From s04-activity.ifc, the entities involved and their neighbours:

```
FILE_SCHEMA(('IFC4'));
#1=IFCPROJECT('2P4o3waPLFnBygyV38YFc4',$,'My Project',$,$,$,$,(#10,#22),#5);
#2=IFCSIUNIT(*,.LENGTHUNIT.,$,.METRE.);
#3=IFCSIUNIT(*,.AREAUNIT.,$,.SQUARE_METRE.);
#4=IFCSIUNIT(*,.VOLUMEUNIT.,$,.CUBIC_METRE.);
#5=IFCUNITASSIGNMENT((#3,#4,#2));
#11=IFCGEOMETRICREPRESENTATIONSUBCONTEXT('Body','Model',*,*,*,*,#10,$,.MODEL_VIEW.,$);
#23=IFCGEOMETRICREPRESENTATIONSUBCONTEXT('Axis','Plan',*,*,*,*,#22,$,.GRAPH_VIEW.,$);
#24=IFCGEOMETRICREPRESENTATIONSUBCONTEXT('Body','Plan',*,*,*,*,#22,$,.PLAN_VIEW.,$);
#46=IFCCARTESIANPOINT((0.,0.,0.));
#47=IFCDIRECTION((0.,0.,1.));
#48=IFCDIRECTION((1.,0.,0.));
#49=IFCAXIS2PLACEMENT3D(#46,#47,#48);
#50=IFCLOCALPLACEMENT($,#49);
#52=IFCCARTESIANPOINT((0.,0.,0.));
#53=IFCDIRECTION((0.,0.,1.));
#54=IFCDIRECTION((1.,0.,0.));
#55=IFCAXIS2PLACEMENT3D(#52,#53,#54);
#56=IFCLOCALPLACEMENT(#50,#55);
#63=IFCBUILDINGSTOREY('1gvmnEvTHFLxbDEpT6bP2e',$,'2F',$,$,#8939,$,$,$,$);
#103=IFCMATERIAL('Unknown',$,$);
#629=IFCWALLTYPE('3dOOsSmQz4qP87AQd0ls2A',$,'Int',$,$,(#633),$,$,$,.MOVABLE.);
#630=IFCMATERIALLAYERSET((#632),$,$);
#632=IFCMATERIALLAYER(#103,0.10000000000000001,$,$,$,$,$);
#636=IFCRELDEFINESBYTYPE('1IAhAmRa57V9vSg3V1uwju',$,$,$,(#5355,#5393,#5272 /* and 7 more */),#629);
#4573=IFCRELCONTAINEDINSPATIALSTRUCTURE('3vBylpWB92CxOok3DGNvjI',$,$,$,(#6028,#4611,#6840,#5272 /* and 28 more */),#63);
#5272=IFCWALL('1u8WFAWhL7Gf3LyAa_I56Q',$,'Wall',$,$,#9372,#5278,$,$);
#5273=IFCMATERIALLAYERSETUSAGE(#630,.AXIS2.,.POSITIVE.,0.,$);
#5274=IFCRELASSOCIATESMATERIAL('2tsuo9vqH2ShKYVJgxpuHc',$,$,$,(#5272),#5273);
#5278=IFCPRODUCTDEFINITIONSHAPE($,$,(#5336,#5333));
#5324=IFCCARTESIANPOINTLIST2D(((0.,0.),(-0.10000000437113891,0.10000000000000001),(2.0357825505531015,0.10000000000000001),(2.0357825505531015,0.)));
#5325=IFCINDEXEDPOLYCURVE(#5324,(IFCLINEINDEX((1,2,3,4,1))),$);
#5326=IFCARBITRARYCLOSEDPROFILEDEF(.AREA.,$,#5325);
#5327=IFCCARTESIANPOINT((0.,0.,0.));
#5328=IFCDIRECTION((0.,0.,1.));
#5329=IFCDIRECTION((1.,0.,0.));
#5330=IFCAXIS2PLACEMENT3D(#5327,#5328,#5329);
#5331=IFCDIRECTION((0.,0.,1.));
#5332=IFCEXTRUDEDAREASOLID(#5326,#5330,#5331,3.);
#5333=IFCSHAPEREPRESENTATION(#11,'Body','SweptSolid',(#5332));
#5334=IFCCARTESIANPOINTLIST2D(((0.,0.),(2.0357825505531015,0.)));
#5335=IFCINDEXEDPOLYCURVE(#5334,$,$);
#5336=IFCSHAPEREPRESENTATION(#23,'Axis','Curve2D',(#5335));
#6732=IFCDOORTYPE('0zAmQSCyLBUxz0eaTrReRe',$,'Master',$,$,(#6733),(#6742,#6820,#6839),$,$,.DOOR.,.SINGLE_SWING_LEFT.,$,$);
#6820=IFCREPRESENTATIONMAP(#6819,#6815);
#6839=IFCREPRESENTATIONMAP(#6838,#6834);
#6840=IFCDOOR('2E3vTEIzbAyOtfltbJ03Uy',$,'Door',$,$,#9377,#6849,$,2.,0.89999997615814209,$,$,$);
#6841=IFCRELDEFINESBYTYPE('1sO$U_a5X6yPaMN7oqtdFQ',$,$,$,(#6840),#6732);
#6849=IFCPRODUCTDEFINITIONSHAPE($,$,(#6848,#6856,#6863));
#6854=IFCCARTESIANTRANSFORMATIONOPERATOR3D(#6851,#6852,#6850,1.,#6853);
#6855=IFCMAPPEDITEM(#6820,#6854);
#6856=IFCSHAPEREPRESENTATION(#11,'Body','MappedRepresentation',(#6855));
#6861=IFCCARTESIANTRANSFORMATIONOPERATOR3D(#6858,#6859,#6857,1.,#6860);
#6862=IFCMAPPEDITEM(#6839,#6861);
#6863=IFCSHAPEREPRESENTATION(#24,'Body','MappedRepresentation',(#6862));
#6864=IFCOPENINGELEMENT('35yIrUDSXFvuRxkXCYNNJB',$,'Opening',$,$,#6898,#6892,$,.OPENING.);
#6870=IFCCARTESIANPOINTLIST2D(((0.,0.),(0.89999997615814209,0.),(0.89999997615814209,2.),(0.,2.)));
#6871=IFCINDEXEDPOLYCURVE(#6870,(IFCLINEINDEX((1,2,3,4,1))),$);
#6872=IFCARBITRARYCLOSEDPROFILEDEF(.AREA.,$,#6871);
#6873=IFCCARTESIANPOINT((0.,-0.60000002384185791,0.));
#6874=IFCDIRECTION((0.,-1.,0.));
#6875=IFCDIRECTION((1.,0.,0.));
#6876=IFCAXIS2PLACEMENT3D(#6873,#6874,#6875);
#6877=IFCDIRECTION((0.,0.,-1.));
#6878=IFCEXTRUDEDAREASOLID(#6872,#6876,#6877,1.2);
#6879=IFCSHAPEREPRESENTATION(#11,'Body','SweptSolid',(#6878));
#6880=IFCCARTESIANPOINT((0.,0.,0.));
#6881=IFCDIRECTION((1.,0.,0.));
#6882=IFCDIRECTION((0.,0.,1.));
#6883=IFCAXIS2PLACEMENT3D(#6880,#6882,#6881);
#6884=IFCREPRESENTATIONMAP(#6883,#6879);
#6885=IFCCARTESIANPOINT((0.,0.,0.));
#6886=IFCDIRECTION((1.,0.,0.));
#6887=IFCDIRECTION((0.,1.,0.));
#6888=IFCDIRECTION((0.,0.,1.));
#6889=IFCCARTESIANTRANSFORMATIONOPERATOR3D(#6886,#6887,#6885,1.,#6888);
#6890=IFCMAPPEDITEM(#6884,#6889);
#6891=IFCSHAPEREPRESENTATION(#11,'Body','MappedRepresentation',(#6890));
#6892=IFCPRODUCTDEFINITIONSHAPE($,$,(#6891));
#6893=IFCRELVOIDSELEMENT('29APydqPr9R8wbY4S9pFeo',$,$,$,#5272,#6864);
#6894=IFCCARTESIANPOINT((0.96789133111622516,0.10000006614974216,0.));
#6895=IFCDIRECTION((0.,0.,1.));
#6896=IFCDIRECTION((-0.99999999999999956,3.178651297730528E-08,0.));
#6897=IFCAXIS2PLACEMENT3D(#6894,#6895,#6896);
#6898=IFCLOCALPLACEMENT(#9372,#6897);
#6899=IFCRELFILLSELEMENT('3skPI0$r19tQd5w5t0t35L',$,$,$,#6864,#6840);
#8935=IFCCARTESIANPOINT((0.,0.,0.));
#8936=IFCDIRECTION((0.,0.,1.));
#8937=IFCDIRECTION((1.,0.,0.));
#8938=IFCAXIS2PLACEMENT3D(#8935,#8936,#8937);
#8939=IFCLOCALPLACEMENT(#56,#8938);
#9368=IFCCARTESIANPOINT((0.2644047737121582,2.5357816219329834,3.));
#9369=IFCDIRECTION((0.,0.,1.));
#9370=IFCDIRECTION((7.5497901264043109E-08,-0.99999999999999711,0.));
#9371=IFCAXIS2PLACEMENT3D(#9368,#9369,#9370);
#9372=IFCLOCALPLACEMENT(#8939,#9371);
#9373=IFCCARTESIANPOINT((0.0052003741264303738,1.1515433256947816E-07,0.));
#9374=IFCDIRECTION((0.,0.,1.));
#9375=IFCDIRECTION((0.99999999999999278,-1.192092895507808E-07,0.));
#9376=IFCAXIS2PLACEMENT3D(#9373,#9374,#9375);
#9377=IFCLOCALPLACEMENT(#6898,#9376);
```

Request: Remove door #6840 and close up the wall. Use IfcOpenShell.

```python
import ifcopenshell
import ifcopenshell.api.feature
import ifcopenshell.api.root
import ifcopenshell.geom
import ifcopenshell.util.shape

model = ifcopenshell.open("s04-activity.ifc")
settings = ifcopenshell.geom.settings()


def volume(element):
    """Net volume in cubic metres, openings subtracted."""
    shape = ifcopenshell.geom.create_shape(settings, element)
    return ifcopenshell.util.shape.get_volume(shape.geometry)


door = model.by_guid("2E3vTEIzbAyOtfltbJ03Uy")
opening = door.FillsVoids[0].RelatingOpeningElement
wall = opening.VoidsElements[0].RelatingBuildingElement
before = volume(wall)

ifcopenshell.api.root.remove_product(model, product=door)
ifcopenshell.api.feature.remove_feature(model, feature=opening)

after = volume(wall)

print(f"wall volume {before:.3f} -> {after:.3f} m3")

model.write("s04-activity_v2.ifc")
```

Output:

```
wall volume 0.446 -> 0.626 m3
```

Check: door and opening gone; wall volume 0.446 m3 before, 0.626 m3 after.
